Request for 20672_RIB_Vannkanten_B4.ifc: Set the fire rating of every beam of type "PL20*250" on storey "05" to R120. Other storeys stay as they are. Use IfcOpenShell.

First a look at what the model holds.

```python
import ifcopenshell
import ifcopenshell.util.element

model = ifcopenshell.open("20672_RIB_Vannkanten_B4.ifc")
print(model.schema)
storey = next(s for s in model.by_type("IfcBuildingStorey") if s.Name == "05")
beams = [e for e in ifcopenshell.util.element.get_decomposition(storey) if e.is_a("IfcBeam")]
seen = {}
for e in beams:
    element_type = ifcopenshell.util.element.get_type(e)
    key = (element_type.Name if element_type != e and element_type else None, ifcopenshell.util.element.get_pset(e, "Pset_BeamCommon", "FireRating"))
    seen[key] = seen.get(key, 0) + 1
for (name, value), count in sorted(seen.items(), key=str):
    print(count, "x", name, "|", value)
```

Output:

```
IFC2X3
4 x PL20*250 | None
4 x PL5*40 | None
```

```python
import ifcopenshell
import ifcopenshell.api.pset
import ifcopenshell.util.element

model = ifcopenshell.open("20672_RIB_Vannkanten_B4.ifc")

storey = next(s for s in model.by_type("IfcBuildingStorey") if s.Name == "05")
beams = [e for e in ifcopenshell.util.element.get_decomposition(storey) if e.is_a("IfcBeam")]

count = 0
for e in beams:
    element_type = ifcopenshell.util.element.get_type(e)
    if element_type in (None, e) or element_type.Name != "PL20*250":
        continue
    # add_pset returns the element's existing set when there is one.
    pset = ifcopenshell.api.pset.add_pset(model, product=e, name="Pset_BeamCommon")
    ifcopenshell.api.pset.edit_pset(model, pset=pset, properties={"FireRating": "R120"})
    count += 1

print(count, "beams updated")

model.write("20672_RIB_Vannkanten_B4-out.ifc")
```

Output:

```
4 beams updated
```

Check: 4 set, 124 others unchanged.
